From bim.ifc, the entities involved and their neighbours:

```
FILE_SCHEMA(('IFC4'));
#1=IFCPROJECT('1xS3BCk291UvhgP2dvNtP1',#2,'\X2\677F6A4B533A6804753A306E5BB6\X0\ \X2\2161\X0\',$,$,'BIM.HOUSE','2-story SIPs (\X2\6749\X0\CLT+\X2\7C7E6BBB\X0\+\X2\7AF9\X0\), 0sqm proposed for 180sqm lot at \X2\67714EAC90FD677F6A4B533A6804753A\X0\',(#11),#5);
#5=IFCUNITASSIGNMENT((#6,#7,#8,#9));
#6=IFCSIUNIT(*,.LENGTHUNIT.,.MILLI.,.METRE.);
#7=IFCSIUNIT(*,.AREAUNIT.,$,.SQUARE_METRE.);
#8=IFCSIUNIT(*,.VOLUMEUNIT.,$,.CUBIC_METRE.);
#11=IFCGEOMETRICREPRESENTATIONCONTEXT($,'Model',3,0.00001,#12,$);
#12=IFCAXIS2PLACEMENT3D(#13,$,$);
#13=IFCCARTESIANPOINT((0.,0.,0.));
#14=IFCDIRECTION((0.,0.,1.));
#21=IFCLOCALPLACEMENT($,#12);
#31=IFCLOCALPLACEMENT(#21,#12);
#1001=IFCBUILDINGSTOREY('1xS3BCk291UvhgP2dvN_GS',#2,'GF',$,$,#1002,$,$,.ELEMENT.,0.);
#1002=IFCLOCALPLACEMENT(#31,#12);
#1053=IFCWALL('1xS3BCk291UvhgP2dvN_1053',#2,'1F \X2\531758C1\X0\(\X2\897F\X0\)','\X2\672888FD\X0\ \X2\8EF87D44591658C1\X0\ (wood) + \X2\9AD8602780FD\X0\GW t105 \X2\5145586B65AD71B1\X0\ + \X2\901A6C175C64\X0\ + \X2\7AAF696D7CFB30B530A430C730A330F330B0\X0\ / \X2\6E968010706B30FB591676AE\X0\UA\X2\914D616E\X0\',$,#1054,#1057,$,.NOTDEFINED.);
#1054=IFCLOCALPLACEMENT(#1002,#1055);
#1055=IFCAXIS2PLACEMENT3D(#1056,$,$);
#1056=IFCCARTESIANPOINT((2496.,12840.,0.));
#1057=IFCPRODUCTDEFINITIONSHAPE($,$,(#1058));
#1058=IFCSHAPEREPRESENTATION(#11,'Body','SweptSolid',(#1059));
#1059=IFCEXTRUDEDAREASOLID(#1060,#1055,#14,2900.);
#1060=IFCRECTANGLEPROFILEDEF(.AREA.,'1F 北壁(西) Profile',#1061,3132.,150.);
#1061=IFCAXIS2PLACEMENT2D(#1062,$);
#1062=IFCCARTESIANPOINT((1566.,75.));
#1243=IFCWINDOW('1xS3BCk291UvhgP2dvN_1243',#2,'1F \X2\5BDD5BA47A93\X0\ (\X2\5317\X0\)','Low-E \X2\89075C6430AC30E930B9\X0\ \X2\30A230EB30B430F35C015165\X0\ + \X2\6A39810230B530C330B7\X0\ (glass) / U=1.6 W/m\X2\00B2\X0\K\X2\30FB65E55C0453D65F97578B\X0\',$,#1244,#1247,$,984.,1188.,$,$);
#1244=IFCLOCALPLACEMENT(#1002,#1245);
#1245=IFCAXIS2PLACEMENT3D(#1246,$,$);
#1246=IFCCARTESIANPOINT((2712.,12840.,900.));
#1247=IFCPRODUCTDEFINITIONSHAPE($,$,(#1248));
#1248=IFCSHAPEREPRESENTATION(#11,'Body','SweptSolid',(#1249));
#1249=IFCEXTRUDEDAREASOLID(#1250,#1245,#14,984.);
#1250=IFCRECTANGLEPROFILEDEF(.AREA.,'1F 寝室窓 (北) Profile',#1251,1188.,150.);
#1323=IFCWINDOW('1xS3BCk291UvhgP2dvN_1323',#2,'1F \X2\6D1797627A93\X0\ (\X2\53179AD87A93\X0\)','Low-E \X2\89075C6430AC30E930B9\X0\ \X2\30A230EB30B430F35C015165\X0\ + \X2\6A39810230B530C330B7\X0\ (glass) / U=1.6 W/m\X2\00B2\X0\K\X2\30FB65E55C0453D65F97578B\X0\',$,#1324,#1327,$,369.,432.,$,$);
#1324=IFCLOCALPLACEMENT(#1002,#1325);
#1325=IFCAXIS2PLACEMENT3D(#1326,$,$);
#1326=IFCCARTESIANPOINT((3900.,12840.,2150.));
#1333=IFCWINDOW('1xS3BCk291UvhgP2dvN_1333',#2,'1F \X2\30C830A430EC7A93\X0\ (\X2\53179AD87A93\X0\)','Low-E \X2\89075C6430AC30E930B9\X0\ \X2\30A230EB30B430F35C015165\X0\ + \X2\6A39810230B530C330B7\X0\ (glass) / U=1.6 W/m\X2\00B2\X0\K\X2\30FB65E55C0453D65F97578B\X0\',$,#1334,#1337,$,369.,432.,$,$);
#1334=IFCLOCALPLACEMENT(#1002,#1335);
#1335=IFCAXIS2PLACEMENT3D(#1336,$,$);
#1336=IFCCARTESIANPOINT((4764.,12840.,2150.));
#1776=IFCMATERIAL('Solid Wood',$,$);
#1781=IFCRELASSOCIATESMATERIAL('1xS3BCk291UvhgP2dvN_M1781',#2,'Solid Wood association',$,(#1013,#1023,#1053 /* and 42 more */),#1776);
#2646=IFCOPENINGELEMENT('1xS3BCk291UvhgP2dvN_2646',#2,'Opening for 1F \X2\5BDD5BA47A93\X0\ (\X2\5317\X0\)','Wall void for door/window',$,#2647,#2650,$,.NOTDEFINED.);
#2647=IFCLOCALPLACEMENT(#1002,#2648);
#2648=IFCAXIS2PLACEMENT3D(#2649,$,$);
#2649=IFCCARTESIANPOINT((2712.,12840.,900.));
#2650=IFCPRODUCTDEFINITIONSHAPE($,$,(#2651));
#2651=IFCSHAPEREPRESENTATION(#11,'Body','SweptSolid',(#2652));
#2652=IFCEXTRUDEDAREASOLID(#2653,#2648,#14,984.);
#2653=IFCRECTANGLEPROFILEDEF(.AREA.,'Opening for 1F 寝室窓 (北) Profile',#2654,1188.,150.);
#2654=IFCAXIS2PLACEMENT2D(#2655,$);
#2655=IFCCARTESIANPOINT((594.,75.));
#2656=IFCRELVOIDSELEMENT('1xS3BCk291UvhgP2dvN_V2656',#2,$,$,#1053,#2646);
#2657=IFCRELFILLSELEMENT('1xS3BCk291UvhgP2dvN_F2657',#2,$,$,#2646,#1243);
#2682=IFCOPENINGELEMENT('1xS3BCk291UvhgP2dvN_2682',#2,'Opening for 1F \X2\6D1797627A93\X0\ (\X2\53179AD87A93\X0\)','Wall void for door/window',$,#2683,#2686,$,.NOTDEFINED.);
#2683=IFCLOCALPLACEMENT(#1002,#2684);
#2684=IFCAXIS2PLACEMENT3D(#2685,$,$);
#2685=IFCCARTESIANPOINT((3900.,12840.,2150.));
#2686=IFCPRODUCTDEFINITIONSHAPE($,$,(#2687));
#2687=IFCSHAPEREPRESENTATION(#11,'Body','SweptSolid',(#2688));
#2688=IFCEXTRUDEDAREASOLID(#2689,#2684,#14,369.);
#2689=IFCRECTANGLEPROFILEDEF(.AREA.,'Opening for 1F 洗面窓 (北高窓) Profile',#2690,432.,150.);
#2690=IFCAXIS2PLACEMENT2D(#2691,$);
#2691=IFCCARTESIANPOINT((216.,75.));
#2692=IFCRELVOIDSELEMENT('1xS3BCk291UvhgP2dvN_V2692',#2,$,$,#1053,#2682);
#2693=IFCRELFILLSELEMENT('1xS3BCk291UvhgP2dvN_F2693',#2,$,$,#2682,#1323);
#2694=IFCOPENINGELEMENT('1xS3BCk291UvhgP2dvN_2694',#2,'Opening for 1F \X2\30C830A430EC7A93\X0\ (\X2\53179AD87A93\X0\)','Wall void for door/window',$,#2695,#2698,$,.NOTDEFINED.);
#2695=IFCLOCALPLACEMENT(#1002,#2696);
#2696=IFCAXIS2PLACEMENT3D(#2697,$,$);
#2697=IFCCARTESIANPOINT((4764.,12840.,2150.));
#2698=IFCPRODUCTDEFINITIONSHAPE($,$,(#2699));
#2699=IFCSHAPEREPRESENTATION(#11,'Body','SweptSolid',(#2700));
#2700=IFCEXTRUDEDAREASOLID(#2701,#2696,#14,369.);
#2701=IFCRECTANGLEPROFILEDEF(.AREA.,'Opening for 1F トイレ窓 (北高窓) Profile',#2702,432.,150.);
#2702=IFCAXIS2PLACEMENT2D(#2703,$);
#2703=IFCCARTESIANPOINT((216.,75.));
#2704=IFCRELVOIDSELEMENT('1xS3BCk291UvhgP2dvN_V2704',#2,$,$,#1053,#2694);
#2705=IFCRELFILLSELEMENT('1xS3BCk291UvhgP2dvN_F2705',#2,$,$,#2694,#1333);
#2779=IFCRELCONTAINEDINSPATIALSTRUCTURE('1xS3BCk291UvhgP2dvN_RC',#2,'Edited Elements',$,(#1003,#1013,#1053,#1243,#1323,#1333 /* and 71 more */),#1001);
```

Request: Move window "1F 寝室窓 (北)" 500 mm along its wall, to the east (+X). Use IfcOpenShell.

```python
import ifcopenshell
import ifcopenshell.api.geometry
import ifcopenshell.util.placement

model = ifcopenshell.open("bim.ifc")

window = model.by_guid("1xS3BCk291UvhgP2dvN_1243")
opening = window.FillsVoids[0].RelatingOpeningElement
wall = opening.VoidsElements[0].RelatingBuildingElement

wall_matrix = ifcopenshell.util.placement.get_local_placement(wall.ObjectPlacement)
shift = wall_matrix[:3, 0] * 500.0
before = ifcopenshell.util.placement.get_local_placement(window.ObjectPlacement)[:3, 3].copy()

# The window is not placed relative to its opening, so move both.
for product in (opening, window):
    matrix = ifcopenshell.util.placement.get_local_placement(product.ObjectPlacement)
    matrix[:3, 3] += shift
    ifcopenshell.api.geometry.edit_object_placement(model, product=product, matrix=matrix, is_si=False)

after = ifcopenshell.util.placement.get_local_placement(window.ObjectPlacement)[:3, 3]
print("window moved by", (after - before).round(3) + 0.0)

model.write("bim_rev.ifc")
```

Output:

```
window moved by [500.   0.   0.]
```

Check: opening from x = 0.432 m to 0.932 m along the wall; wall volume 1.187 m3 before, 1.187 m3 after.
